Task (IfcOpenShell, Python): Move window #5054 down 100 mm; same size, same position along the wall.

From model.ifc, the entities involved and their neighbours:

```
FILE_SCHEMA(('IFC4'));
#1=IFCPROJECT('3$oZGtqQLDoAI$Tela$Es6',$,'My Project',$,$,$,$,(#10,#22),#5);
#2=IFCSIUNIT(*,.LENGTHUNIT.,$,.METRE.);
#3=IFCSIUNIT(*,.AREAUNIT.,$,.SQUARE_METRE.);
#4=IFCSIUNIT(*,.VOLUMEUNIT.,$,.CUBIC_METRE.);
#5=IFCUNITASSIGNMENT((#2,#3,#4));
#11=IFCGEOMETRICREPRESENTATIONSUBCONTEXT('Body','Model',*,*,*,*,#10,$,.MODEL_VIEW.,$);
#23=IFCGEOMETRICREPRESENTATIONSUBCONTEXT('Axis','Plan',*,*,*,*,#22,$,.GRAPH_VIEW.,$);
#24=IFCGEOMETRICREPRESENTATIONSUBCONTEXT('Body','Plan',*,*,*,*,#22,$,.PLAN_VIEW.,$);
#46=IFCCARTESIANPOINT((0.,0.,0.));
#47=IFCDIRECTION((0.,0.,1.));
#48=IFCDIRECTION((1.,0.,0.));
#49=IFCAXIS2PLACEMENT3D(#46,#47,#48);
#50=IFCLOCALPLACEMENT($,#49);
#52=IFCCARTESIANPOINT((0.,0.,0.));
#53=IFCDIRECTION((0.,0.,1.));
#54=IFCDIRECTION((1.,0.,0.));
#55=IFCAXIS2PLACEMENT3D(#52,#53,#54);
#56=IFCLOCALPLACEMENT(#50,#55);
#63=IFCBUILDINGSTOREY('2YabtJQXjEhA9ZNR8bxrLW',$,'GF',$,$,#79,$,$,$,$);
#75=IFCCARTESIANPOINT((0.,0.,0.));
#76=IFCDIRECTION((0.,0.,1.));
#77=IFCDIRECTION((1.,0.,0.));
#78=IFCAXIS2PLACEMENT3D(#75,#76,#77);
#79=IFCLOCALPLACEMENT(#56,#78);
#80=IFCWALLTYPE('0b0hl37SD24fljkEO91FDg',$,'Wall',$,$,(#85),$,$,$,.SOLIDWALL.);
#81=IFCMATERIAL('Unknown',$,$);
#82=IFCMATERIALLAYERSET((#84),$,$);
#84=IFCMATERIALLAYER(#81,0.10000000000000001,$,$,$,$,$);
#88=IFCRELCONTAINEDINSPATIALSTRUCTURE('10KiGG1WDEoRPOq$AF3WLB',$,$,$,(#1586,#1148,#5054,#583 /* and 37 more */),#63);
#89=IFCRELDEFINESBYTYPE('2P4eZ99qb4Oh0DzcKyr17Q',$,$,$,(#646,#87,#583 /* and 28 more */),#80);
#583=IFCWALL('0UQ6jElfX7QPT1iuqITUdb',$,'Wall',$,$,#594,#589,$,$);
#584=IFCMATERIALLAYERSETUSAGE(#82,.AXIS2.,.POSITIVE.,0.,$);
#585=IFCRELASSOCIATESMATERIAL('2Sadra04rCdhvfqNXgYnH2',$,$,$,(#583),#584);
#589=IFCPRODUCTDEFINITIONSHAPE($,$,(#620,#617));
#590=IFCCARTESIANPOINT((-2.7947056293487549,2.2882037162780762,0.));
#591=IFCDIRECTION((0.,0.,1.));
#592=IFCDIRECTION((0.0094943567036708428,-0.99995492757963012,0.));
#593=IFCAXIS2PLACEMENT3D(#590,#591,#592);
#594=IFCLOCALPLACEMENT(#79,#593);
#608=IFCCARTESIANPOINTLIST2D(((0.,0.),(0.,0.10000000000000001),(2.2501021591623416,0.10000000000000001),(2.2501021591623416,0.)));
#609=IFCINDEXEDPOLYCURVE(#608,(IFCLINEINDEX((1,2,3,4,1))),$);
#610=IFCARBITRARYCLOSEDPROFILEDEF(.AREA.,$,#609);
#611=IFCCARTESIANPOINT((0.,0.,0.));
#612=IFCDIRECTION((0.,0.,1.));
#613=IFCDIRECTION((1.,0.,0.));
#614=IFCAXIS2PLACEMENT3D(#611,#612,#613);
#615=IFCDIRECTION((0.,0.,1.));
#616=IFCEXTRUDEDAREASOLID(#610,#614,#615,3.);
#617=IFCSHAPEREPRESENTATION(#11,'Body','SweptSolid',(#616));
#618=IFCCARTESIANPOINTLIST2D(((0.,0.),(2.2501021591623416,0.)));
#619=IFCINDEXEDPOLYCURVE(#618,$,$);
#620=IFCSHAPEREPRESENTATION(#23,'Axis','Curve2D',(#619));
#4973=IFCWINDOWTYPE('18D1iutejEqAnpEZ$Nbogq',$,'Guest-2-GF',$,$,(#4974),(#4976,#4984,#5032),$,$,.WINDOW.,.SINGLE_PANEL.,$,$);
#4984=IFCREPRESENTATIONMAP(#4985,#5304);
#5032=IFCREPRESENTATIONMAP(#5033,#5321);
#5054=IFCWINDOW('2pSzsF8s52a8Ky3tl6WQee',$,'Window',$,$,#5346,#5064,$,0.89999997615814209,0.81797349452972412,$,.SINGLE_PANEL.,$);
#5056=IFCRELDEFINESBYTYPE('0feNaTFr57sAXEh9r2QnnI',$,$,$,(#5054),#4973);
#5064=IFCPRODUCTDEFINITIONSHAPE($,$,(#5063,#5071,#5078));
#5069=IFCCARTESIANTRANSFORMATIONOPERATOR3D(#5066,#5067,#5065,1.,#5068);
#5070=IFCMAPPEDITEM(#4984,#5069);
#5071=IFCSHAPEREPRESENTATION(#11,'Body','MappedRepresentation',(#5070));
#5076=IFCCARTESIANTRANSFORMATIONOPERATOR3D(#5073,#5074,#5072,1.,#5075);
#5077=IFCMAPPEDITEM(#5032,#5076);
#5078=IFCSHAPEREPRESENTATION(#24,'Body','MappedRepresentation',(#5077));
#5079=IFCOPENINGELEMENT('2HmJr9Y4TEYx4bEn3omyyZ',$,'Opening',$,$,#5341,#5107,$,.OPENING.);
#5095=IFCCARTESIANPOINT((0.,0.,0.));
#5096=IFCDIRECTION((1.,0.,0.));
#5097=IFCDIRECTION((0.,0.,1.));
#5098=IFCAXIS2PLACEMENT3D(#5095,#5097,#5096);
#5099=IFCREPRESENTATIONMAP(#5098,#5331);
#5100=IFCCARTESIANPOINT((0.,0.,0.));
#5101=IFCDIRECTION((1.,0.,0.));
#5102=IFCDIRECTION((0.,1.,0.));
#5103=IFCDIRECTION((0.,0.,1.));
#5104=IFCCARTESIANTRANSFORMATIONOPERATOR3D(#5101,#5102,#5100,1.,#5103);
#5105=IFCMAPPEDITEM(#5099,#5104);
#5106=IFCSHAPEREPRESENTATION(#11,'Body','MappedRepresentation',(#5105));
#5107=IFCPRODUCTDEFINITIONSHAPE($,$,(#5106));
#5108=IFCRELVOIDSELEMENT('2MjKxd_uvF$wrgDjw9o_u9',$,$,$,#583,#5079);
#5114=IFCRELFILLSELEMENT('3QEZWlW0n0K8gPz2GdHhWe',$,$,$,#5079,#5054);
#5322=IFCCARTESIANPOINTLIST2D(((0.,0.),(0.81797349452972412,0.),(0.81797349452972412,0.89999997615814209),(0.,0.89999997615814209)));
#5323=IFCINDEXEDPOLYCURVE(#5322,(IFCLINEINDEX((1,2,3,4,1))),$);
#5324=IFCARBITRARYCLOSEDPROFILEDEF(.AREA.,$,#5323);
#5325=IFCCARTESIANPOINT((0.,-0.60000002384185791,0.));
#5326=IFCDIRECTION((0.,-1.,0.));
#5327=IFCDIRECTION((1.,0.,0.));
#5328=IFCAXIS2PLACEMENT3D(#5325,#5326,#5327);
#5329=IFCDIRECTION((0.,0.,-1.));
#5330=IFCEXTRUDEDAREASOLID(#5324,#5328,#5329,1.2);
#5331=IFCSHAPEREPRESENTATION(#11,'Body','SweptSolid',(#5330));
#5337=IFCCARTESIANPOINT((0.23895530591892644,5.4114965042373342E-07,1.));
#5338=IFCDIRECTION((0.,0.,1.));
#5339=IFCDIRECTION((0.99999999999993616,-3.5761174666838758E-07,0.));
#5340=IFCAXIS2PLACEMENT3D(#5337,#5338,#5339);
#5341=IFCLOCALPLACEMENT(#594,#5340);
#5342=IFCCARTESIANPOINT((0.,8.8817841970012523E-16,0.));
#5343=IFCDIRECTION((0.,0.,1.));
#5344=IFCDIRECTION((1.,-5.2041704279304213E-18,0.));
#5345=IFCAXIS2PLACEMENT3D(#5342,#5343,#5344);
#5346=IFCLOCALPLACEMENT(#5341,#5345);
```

```python
import numpy as np
import ifcopenshell
import ifcopenshell.api.geometry
import ifcopenshell.util.placement
import ifcopenshell.util.unit

model = ifcopenshell.open("model.ifc")
unit_scale = ifcopenshell.util.unit.calculate_unit_scale(model)

window = model.by_guid("2pSzsF8s52a8Ky3tl6WQee")
opening = window.FillsVoids[0].RelatingOpeningElement
dz = -0.1 / unit_scale

shift = np.array([0.0, 0.0, dz])
# The window is placed relative to its opening, so it follows when the opening moves.
matrix = ifcopenshell.util.placement.get_local_placement(opening.ObjectPlacement)
matrix[:3, 3] += shift
ifcopenshell.api.geometry.edit_object_placement(
    model, product=opening, matrix=matrix, is_si=False, should_transform_children=True
)

print(f"moved by {dz * unit_scale:+.3f} m")

model.write("model_edited.ifc")
```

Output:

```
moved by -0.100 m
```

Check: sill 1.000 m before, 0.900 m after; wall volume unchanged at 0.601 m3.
